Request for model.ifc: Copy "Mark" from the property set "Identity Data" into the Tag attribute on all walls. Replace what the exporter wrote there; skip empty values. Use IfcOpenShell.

First a look at what the model holds.

```python
import ifcopenshell
import ifcopenshell.util.element

model = ifcopenshell.open("model.ifc")
print(model.schema)
walls = model.by_type("IfcWall")
print(len(walls), "walls")
for e in walls[:8]:
    source = ifcopenshell.util.element.get_pset(e, "Identity Data", "Mark")
    target = e.Tag
    print(e.id(), repr(source), repr(target), sep=" | ")
```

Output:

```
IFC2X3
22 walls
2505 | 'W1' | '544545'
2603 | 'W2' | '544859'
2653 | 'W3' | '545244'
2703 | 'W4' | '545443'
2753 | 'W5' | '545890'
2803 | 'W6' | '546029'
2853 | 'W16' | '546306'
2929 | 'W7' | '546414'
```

```python
import ifcopenshell
import ifcopenshell.util.element

model = ifcopenshell.open("model.ifc")

count = 0
for e in model.by_type("IfcWall"):
    value = ifcopenshell.util.element.get_pset(e, "Identity Data", "Mark")
    current = e.Tag
    if not value or not value.strip() or current == value:
        continue
    e.Tag = value
    count += 1

print(count, "walls updated")

model.write("model_updated.ifc")
```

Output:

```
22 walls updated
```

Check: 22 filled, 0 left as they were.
